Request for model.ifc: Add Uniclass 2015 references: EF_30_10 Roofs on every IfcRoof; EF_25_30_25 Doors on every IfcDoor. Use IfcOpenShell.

First a look at what the model holds.

```python
import ifcopenshell

model = ifcopenshell.open("model.ifc")
print(model.schema)
print("classifications:", [c.Name for c in model.by_type("IfcClassification")])
for ifc_class in ("IfcDoor", "IfcRoof", "IfcStair", "IfcWall", "IfcWindow"):
    print(ifc_class, len(model.by_type(ifc_class)))
```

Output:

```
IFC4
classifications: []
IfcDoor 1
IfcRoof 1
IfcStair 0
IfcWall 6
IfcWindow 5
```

```python
import ifcopenshell
import ifcopenshell.api.classification

model = ifcopenshell.open("model.ifc")

system = ifcopenshell.api.classification.add_classification(model, classification="Uniclass 2015")

codes = {
    "IfcRoof": ("EF_30_10", "Roofs"),
    "IfcDoor": ("EF_25_30_25", "Doors"),
}
for ifc_class, (code, name) in codes.items():
    products = model.by_type(ifc_class)
    ifcopenshell.api.classification.add_reference(
        model, products=products, classification=system, identification=code, name=name
    )
    print(code, len(products))

model.write("model_rev.ifc")
```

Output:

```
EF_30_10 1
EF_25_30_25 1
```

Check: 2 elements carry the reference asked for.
